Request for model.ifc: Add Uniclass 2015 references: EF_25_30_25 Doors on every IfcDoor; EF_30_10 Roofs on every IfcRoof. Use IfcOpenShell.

First a look at what the model holds.

```python
import ifcopenshell

model = ifcopenshell.open("model.ifc")
print(model.schema)
print("classifications:", [c.Name for c in model.by_type("IfcClassification")])
for ifc_class in ("IfcDoor", "IfcRoof", "IfcStair", "IfcWall", "IfcWindow"):
    print(ifc_class, len(model.by_type(ifc_class)))
```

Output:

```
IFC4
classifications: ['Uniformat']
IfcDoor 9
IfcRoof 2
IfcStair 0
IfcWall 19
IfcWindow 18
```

```python
import ifcopenshell
import ifcopenshell.api.classification

model = ifcopenshell.open("model.ifc")

system = ifcopenshell.api.classification.add_classification(model, classification="Uniclass 2015")

codes = {
    "IfcDoor": ("EF_25_30_25", "Doors"),
    "IfcRoof": ("EF_30_10", "Roofs"),
}
for ifc_class, (code, name) in codes.items():
    products = model.by_type(ifc_class)
    ifcopenshell.api.classification.add_reference(
        model, products=products, classification=system, identification=code, name=name
    )
    print(code, len(products))

model.write("model_v2.ifc")
```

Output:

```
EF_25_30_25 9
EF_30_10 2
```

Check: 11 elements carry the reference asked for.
